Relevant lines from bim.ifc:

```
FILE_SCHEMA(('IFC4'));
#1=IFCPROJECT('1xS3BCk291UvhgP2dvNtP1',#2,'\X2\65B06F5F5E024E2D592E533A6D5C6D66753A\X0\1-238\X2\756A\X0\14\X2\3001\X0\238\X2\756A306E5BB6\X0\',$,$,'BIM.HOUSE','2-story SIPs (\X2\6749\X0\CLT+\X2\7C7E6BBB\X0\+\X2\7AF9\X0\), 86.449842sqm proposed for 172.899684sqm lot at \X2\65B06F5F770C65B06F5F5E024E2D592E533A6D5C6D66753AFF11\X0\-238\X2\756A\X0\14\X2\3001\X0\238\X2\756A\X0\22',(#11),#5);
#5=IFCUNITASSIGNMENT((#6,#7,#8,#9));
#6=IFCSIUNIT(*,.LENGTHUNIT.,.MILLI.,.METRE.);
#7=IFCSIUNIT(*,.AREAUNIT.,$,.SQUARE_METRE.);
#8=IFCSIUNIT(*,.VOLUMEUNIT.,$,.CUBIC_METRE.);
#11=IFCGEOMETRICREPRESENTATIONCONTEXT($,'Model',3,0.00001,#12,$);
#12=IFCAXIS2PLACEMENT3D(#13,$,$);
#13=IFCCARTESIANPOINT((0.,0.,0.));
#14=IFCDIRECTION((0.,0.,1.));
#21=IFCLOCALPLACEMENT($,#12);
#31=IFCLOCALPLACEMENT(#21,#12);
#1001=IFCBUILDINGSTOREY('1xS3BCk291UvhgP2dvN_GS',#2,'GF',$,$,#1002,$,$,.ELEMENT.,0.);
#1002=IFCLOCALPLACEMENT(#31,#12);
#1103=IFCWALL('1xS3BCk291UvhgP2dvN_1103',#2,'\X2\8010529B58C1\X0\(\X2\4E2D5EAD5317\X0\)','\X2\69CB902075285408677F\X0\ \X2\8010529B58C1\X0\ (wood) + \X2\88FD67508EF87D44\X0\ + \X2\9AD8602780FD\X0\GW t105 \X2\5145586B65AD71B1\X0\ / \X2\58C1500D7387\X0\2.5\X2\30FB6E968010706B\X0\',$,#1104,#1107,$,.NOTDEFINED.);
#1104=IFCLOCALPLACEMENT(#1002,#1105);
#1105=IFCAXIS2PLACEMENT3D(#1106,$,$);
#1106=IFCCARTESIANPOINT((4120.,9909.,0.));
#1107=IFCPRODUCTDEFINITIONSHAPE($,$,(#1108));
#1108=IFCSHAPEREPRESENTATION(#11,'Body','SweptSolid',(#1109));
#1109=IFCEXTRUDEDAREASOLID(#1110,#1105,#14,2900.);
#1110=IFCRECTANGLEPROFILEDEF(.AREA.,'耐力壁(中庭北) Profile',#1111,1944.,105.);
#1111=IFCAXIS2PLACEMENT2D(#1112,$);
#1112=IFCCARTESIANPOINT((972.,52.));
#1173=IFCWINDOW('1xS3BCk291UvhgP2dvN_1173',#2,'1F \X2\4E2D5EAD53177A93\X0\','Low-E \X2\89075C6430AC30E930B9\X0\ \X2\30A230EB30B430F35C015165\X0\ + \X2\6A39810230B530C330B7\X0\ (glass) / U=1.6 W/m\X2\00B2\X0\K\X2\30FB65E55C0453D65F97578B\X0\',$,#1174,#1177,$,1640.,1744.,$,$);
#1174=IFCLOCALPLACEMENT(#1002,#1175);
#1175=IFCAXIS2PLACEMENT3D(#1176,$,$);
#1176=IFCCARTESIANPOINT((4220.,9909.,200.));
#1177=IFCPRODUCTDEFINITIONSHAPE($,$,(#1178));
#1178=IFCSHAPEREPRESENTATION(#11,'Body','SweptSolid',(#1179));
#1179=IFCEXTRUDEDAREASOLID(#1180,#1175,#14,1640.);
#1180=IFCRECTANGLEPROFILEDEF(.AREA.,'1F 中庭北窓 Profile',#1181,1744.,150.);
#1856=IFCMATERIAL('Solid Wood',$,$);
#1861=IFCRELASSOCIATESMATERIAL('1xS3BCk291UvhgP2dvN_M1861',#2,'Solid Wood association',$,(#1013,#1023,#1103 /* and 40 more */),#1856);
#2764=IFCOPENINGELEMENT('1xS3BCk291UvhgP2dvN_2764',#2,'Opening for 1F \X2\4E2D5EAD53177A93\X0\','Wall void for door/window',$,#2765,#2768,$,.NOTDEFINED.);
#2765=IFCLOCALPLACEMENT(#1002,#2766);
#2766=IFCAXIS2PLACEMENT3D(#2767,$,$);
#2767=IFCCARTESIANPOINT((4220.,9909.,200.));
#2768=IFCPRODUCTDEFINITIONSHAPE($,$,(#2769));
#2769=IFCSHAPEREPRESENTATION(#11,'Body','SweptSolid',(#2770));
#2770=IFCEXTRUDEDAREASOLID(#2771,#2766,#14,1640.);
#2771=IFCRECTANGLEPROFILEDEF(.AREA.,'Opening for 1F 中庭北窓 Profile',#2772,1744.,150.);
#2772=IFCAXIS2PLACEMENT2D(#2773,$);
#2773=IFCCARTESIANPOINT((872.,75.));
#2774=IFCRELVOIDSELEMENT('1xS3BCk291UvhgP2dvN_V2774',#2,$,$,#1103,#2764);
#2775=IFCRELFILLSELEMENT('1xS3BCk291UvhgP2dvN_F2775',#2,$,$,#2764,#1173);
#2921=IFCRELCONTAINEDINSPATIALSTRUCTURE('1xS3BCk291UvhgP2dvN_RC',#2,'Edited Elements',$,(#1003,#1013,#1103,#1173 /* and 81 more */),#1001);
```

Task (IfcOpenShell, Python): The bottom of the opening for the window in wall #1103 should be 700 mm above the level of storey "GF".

```python
import numpy as np
import ifcopenshell
import ifcopenshell.api.geometry
import ifcopenshell.geom
import ifcopenshell.util.element
import ifcopenshell.util.placement
import ifcopenshell.util.shape
import ifcopenshell.util.unit

model = ifcopenshell.open("bim.ifc")
unit_scale = ifcopenshell.util.unit.calculate_unit_scale(model)

window = model.by_guid("1xS3BCk291UvhgP2dvN_1173")
opening = window.FillsVoids[0].RelatingOpeningElement
storey = ifcopenshell.util.element.get_container(window, ifc_class="IfcBuildingStorey")
level = ifcopenshell.util.placement.get_local_placement(storey.ObjectPlacement)[2, 3]

# The opening's origin need not be at the sill, so measure its lowest point.
shape = ifcopenshell.geom.create_shape(ifcopenshell.geom.settings(), opening)
bottom = ifcopenshell.util.shape.get_shape_bottom_elevation(shape, shape.geometry) / unit_scale
dz = level + 700.0 - bottom

shift = np.array([0.0, 0.0, dz])
# The window is not placed relative to its opening, so move both.
for product in (opening, window):
    matrix = ifcopenshell.util.placement.get_local_placement(product.ObjectPlacement)
    matrix[:3, 3] += shift
    ifcopenshell.api.geometry.edit_object_placement(model, product=product, matrix=matrix, is_si=False)

print(f"moved by {dz * unit_scale:+.3f} m")

model.write("bim_rev.ifc")
```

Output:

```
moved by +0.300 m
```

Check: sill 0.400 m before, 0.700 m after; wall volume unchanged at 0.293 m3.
